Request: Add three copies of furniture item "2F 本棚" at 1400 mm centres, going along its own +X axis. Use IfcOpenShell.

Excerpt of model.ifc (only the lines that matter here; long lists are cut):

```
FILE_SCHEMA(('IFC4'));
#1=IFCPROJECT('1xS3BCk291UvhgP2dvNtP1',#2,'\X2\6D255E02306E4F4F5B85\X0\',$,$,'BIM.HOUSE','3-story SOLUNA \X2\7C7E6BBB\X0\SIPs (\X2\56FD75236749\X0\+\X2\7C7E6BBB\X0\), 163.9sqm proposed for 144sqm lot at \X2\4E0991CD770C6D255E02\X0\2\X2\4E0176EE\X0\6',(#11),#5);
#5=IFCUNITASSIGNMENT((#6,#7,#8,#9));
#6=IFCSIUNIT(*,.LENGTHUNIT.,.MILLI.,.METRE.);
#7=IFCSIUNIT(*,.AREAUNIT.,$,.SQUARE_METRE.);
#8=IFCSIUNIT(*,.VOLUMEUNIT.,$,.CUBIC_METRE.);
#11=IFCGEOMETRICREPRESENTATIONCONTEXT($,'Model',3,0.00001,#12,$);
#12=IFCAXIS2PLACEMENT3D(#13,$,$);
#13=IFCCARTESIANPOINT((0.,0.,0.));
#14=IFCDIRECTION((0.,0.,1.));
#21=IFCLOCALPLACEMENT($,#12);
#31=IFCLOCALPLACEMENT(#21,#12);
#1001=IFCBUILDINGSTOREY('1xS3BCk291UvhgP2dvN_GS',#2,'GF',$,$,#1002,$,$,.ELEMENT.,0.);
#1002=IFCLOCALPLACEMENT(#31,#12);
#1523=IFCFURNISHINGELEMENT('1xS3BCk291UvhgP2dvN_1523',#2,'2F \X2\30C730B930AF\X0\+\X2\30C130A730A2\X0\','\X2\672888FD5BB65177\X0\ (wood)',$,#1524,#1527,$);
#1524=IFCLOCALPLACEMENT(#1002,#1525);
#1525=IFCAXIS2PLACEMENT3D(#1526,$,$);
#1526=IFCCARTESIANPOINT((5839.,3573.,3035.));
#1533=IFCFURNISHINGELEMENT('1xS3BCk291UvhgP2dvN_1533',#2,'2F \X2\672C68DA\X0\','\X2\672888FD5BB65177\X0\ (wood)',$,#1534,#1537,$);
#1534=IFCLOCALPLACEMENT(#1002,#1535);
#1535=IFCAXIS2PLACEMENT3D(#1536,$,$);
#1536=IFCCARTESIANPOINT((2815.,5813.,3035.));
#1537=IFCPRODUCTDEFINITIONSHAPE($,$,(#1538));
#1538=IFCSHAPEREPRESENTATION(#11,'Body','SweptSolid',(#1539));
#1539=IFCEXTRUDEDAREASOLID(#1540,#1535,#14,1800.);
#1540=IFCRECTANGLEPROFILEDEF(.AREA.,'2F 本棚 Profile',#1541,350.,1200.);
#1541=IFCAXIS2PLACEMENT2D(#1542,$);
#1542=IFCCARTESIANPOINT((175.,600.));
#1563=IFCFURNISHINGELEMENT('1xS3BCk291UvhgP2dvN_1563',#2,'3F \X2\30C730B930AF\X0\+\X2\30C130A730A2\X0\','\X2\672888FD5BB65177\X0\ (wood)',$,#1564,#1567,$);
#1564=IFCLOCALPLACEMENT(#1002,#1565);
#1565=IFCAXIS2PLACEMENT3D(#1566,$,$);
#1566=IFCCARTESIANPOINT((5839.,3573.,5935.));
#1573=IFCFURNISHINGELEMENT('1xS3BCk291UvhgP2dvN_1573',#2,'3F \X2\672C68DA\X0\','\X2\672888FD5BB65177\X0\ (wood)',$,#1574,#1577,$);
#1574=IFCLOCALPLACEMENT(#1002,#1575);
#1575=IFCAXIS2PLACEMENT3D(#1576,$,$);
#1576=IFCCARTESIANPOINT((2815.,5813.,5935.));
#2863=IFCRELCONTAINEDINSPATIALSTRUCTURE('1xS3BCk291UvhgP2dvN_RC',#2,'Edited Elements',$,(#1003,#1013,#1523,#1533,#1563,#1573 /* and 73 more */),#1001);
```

```python
import ifcopenshell
import ifcopenshell.api.geometry
import ifcopenshell.api.root
import ifcopenshell.util.element
import ifcopenshell.util.placement

model = ifcopenshell.open("model.ifc")


def reuse_history(source, copy):
    """copy_class also copies each property set's owner history, people and application; keep the originals."""
    for rel in copy.IsDefinedBy:
        if rel.is_a("IfcRelDefinesByProperties") and (history := rel.RelatingPropertyDefinition.OwnerHistory):
            rel.RelatingPropertyDefinition.OwnerHistory = source.OwnerHistory
            ifcopenshell.util.element.remove_deep2(model, history)


source = model.by_guid("1xS3BCk291UvhgP2dvN_1533")
base = ifcopenshell.util.placement.get_local_placement(source.ObjectPlacement)
step = base[:3, 0] * 1400.0

for i in range(1, 4):
    copy = ifcopenshell.api.root.copy_class(model, product=source)
    copy.Representation = ifcopenshell.util.element.copy_deep(
        model, source.Representation, exclude=["IfcGeometricRepresentationContext", "IfcRepresentationMap"]
    )
    reuse_history(source, copy)
    matrix = base.copy()
    matrix[:3, 3] += i * step
    print("added at", matrix[:3, 3].round(3) + 0.0)
    ifcopenshell.api.geometry.edit_object_placement(model, product=copy, matrix=matrix, is_si=False)

model.write("model_rev.ifc")
```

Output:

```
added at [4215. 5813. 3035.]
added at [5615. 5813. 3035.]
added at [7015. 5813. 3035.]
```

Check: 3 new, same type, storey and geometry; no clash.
